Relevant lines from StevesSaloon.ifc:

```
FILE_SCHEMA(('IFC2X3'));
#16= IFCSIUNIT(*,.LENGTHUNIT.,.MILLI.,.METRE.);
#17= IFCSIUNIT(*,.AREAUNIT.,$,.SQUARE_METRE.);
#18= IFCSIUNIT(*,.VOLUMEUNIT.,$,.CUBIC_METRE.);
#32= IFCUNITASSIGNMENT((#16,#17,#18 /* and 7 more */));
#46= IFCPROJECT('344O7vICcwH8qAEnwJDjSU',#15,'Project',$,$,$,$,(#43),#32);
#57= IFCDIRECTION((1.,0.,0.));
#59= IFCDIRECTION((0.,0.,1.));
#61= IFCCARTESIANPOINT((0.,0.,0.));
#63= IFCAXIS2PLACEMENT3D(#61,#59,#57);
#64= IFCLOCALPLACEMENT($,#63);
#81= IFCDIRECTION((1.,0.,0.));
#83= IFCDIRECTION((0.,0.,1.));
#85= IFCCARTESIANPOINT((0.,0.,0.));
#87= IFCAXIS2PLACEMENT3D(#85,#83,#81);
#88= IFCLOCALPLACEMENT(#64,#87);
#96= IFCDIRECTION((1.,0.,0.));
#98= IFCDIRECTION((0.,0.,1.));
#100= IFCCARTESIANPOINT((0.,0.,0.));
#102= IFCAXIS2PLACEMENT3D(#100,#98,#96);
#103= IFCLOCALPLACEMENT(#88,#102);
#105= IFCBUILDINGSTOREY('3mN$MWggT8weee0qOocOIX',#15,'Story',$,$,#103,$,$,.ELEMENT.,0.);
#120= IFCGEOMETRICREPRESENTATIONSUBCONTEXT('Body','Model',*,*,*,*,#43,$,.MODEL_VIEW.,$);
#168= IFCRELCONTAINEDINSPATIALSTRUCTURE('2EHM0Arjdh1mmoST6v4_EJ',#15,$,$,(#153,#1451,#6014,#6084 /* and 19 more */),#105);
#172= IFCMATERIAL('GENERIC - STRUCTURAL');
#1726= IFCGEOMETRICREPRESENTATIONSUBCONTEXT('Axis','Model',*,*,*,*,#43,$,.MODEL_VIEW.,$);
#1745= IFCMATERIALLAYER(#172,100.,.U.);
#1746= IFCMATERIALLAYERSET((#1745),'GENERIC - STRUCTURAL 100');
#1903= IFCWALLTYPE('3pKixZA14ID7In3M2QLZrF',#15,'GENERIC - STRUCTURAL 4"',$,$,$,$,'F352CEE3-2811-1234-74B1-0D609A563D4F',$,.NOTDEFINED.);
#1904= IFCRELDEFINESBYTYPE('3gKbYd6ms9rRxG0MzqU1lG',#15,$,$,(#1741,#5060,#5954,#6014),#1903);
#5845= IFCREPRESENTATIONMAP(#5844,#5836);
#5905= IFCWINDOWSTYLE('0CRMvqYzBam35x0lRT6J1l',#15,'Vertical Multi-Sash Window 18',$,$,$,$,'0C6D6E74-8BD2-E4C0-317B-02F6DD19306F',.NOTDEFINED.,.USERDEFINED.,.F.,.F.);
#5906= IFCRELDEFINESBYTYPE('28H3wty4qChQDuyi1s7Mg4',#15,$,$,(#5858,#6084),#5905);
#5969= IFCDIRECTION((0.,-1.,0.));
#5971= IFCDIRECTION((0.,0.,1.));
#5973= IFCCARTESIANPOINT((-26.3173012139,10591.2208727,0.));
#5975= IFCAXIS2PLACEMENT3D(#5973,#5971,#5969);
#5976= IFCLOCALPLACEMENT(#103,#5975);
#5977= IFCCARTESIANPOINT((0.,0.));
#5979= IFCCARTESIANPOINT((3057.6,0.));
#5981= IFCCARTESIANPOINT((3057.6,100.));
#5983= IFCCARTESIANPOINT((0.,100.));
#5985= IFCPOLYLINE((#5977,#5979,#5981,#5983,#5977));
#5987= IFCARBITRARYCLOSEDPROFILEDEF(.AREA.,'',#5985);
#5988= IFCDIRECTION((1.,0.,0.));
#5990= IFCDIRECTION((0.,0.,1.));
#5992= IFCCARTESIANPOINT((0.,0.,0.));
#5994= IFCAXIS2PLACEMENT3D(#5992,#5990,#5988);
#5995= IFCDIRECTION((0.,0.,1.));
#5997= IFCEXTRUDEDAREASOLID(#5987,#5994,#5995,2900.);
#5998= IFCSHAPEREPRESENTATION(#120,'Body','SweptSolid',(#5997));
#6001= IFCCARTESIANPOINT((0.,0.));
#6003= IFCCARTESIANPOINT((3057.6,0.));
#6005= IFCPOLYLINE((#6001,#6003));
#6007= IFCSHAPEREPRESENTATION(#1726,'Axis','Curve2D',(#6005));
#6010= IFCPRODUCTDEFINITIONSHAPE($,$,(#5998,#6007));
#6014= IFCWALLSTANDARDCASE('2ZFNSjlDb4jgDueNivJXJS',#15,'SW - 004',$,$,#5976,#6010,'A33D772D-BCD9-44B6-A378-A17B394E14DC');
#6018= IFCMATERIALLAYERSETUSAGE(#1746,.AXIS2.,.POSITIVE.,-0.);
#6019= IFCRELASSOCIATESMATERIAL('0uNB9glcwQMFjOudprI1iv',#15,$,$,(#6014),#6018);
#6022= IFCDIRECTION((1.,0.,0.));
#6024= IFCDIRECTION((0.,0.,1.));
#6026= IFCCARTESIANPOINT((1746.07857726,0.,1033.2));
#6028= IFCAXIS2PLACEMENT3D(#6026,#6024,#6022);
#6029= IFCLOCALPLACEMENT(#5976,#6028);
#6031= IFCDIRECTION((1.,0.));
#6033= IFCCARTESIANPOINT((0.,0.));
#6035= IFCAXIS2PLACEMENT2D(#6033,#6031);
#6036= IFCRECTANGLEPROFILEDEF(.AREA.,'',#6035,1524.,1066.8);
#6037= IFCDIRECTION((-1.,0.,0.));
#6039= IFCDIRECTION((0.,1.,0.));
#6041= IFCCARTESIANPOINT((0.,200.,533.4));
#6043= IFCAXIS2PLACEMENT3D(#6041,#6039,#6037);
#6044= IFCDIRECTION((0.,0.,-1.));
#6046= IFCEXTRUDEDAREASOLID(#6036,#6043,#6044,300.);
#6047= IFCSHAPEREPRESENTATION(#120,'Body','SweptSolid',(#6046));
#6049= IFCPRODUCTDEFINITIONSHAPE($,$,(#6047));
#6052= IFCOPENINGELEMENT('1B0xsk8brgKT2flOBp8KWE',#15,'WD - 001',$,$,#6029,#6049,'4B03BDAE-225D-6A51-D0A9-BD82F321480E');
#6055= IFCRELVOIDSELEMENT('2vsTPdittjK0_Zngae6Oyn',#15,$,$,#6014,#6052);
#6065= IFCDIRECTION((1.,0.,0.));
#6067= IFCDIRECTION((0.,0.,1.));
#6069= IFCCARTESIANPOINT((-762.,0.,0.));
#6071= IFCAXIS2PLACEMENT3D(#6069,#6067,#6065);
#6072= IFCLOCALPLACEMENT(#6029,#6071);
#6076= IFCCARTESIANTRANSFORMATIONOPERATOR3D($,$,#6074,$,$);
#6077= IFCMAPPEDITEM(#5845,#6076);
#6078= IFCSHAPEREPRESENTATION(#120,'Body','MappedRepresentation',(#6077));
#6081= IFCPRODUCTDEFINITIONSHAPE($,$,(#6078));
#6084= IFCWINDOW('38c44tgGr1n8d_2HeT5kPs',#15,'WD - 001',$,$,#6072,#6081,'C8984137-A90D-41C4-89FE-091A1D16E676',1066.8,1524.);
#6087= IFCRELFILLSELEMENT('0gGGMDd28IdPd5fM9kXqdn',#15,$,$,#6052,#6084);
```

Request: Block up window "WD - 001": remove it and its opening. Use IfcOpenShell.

```python
import ifcopenshell
import ifcopenshell.api.feature
import ifcopenshell.api.root
import ifcopenshell.geom
import ifcopenshell.util.shape

model = ifcopenshell.open("StevesSaloon.ifc")
settings = ifcopenshell.geom.settings()


def volume(element):
    """Net volume in cubic metres, openings subtracted."""
    shape = ifcopenshell.geom.create_shape(settings, element)
    return ifcopenshell.util.shape.get_volume(shape.geometry)


window = model.by_guid("38c44tgGr1n8d_2HeT5kPs")
opening = window.FillsVoids[0].RelatingOpeningElement
wall = opening.VoidsElements[0].RelatingBuildingElement
before = volume(wall)

ifcopenshell.api.root.remove_product(model, product=window)
ifcopenshell.api.feature.remove_feature(model, feature=opening)

after = volume(wall)

print(f"wall volume {before:.3f} -> {after:.3f} m3")

model.write("StevesSaloon_rev.ifc")
```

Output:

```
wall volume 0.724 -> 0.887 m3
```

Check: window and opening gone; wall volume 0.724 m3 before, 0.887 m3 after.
